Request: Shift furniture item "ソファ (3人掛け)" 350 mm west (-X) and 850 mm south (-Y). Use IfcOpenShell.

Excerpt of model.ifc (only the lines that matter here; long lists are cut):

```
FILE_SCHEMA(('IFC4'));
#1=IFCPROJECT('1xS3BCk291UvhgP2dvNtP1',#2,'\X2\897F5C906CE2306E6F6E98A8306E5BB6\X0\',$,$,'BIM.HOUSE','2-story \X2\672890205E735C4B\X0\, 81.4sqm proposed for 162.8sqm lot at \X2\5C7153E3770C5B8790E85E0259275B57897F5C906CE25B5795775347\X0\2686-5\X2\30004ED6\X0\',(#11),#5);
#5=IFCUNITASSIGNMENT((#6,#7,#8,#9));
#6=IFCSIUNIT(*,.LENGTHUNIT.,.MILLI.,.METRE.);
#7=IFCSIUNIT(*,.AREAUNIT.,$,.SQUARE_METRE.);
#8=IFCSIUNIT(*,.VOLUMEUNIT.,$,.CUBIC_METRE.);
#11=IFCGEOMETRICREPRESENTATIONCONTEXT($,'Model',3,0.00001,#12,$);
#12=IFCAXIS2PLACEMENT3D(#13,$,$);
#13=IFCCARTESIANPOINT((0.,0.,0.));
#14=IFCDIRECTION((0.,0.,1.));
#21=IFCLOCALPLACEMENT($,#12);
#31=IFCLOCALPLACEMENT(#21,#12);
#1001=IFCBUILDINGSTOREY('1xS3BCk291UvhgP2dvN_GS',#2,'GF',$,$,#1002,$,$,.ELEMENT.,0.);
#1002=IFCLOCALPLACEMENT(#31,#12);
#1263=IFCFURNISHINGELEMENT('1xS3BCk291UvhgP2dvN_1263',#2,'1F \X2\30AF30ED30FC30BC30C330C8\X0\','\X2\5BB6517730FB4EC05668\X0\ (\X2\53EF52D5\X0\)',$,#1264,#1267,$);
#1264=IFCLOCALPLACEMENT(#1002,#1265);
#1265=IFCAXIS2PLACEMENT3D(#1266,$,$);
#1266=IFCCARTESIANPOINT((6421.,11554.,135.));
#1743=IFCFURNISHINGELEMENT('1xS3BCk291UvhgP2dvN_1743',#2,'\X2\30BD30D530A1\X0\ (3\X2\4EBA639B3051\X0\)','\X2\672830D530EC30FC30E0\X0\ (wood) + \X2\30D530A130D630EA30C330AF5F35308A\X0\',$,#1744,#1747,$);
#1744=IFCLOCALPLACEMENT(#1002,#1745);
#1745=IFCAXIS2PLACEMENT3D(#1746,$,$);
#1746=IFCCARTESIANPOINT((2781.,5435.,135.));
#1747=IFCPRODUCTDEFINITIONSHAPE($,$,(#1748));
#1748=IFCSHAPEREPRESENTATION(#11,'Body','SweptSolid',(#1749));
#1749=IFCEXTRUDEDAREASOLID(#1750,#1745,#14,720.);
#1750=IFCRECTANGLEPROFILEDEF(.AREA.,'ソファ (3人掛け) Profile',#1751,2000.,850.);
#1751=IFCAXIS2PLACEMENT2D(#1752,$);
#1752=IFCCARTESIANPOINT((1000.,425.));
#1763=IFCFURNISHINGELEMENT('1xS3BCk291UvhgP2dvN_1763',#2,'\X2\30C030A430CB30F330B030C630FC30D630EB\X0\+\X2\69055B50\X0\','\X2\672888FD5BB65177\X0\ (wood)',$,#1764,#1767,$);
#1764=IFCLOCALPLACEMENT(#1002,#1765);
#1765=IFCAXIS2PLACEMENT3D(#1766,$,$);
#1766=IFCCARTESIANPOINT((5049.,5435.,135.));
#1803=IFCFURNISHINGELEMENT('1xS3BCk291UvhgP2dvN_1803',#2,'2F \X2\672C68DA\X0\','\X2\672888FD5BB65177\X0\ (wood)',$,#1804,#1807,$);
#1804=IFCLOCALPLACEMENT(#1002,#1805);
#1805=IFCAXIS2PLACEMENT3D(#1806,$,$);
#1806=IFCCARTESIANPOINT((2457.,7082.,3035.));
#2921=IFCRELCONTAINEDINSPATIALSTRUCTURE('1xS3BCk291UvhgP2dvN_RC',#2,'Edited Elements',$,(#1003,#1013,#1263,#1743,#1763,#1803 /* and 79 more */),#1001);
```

```python
import ifcopenshell
import ifcopenshell.api.geometry
import ifcopenshell.util.placement
import ifcopenshell.util.unit

model = ifcopenshell.open("model.ifc")
unit_scale = ifcopenshell.util.unit.calculate_unit_scale(model)

item = model.by_guid("1xS3BCk291UvhgP2dvN_1743")
matrix = ifcopenshell.util.placement.get_local_placement(item.ObjectPlacement)
matrix[0, 3] -= 0.35 / unit_scale
matrix[1, 3] -= 0.85 / unit_scale
ifcopenshell.api.geometry.edit_object_placement(model, product=item, matrix=matrix, is_si=False)

print(ifcopenshell.util.placement.get_local_placement(item.ObjectPlacement).round(3) + 0.0)

model.write("model_updated.ifc")
```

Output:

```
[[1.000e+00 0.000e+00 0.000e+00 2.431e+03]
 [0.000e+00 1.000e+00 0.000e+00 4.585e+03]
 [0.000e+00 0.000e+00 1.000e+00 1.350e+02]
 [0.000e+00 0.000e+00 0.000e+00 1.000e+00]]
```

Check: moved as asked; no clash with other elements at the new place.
